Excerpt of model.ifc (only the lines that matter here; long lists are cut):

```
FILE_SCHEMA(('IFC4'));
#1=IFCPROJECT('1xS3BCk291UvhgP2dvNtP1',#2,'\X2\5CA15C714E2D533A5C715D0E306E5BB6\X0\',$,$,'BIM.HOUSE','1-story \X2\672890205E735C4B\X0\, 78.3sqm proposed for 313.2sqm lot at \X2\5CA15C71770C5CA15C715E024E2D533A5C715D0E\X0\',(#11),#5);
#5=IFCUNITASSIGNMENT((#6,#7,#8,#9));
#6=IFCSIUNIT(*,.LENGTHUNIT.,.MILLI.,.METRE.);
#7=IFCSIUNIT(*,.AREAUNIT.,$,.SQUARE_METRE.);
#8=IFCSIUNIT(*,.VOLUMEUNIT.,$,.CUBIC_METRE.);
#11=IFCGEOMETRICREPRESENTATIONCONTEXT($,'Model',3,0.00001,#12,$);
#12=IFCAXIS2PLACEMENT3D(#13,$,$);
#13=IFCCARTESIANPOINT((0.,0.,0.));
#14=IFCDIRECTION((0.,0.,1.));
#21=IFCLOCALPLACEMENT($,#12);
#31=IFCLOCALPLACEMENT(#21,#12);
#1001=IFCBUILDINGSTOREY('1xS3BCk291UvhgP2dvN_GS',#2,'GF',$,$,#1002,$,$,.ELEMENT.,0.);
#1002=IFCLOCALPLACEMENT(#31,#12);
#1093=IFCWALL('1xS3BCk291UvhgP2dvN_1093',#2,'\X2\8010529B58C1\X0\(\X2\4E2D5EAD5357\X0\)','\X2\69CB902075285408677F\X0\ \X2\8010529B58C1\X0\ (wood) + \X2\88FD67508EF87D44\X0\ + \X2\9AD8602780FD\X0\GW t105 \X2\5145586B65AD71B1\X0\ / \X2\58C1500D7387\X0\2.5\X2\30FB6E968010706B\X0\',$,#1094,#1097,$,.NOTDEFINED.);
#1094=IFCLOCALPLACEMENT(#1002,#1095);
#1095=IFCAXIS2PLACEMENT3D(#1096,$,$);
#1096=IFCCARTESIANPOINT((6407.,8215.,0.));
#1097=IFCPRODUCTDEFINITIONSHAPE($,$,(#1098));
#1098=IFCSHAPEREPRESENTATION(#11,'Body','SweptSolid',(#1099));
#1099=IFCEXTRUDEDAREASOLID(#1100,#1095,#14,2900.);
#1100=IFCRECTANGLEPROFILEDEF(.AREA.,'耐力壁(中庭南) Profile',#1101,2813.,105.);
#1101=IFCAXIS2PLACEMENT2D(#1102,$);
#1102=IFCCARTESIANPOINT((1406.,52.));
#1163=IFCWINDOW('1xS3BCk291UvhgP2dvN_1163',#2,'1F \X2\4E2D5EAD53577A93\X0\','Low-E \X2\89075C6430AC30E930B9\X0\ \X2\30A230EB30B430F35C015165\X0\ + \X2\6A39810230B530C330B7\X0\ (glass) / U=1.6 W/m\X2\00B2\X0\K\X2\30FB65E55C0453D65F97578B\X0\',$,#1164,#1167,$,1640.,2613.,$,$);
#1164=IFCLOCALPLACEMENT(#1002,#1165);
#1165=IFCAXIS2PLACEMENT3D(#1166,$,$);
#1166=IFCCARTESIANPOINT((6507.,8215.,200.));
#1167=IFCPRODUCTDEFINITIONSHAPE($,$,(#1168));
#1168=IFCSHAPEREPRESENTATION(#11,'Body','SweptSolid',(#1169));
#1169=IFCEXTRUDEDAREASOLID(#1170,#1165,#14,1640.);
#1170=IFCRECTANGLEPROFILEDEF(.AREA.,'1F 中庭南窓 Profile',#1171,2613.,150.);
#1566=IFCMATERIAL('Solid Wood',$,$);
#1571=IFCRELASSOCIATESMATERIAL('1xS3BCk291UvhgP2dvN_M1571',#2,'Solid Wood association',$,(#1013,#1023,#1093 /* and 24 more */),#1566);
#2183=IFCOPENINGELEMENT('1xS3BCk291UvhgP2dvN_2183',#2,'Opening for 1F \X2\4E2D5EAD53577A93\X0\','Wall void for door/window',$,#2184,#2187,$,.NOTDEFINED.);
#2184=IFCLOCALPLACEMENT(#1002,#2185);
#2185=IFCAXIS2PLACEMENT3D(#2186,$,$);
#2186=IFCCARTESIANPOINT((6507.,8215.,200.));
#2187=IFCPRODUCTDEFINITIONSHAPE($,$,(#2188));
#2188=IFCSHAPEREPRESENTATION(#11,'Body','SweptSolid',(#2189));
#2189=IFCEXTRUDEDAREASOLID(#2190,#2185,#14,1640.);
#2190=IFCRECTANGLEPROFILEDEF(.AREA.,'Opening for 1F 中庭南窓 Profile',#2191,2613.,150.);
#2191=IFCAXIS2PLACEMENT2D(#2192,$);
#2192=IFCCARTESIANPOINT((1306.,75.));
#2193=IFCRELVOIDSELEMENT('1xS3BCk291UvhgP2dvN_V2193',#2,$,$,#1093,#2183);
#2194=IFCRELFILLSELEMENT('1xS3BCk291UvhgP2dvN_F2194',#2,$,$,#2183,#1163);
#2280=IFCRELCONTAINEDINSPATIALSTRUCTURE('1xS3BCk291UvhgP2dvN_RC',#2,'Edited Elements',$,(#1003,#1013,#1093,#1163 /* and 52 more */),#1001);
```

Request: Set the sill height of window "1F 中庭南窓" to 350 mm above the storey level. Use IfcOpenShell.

```python
import numpy as np
import ifcopenshell
import ifcopenshell.api.geometry
import ifcopenshell.geom
import ifcopenshell.util.element
import ifcopenshell.util.placement
import ifcopenshell.util.shape
import ifcopenshell.util.unit

model = ifcopenshell.open("model.ifc")
unit_scale = ifcopenshell.util.unit.calculate_unit_scale(model)

window = model.by_id(1163)
opening = window.FillsVoids[0].RelatingOpeningElement
storey = ifcopenshell.util.element.get_container(window, ifc_class="IfcBuildingStorey")
level = ifcopenshell.util.placement.get_local_placement(storey.ObjectPlacement)[2, 3]

# The opening's origin need not be at the sill, so measure its lowest point.
shape = ifcopenshell.geom.create_shape(ifcopenshell.geom.settings(), opening)
bottom = ifcopenshell.util.shape.get_shape_bottom_elevation(shape, shape.geometry) / unit_scale
dz = level + 350.0 - bottom

shift = np.array([0.0, 0.0, dz])
# The window is not placed relative to its opening, so move both.
for product in (opening, window):
    matrix = ifcopenshell.util.placement.get_local_placement(product.ObjectPlacement)
    matrix[:3, 3] += shift
    ifcopenshell.api.geometry.edit_object_placement(model, product=product, matrix=matrix, is_si=False)

print(f"moved by {dz * unit_scale:+.3f} m")

model.write("model-out.ifc")
```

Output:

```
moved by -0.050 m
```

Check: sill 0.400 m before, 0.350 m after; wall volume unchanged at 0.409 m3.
